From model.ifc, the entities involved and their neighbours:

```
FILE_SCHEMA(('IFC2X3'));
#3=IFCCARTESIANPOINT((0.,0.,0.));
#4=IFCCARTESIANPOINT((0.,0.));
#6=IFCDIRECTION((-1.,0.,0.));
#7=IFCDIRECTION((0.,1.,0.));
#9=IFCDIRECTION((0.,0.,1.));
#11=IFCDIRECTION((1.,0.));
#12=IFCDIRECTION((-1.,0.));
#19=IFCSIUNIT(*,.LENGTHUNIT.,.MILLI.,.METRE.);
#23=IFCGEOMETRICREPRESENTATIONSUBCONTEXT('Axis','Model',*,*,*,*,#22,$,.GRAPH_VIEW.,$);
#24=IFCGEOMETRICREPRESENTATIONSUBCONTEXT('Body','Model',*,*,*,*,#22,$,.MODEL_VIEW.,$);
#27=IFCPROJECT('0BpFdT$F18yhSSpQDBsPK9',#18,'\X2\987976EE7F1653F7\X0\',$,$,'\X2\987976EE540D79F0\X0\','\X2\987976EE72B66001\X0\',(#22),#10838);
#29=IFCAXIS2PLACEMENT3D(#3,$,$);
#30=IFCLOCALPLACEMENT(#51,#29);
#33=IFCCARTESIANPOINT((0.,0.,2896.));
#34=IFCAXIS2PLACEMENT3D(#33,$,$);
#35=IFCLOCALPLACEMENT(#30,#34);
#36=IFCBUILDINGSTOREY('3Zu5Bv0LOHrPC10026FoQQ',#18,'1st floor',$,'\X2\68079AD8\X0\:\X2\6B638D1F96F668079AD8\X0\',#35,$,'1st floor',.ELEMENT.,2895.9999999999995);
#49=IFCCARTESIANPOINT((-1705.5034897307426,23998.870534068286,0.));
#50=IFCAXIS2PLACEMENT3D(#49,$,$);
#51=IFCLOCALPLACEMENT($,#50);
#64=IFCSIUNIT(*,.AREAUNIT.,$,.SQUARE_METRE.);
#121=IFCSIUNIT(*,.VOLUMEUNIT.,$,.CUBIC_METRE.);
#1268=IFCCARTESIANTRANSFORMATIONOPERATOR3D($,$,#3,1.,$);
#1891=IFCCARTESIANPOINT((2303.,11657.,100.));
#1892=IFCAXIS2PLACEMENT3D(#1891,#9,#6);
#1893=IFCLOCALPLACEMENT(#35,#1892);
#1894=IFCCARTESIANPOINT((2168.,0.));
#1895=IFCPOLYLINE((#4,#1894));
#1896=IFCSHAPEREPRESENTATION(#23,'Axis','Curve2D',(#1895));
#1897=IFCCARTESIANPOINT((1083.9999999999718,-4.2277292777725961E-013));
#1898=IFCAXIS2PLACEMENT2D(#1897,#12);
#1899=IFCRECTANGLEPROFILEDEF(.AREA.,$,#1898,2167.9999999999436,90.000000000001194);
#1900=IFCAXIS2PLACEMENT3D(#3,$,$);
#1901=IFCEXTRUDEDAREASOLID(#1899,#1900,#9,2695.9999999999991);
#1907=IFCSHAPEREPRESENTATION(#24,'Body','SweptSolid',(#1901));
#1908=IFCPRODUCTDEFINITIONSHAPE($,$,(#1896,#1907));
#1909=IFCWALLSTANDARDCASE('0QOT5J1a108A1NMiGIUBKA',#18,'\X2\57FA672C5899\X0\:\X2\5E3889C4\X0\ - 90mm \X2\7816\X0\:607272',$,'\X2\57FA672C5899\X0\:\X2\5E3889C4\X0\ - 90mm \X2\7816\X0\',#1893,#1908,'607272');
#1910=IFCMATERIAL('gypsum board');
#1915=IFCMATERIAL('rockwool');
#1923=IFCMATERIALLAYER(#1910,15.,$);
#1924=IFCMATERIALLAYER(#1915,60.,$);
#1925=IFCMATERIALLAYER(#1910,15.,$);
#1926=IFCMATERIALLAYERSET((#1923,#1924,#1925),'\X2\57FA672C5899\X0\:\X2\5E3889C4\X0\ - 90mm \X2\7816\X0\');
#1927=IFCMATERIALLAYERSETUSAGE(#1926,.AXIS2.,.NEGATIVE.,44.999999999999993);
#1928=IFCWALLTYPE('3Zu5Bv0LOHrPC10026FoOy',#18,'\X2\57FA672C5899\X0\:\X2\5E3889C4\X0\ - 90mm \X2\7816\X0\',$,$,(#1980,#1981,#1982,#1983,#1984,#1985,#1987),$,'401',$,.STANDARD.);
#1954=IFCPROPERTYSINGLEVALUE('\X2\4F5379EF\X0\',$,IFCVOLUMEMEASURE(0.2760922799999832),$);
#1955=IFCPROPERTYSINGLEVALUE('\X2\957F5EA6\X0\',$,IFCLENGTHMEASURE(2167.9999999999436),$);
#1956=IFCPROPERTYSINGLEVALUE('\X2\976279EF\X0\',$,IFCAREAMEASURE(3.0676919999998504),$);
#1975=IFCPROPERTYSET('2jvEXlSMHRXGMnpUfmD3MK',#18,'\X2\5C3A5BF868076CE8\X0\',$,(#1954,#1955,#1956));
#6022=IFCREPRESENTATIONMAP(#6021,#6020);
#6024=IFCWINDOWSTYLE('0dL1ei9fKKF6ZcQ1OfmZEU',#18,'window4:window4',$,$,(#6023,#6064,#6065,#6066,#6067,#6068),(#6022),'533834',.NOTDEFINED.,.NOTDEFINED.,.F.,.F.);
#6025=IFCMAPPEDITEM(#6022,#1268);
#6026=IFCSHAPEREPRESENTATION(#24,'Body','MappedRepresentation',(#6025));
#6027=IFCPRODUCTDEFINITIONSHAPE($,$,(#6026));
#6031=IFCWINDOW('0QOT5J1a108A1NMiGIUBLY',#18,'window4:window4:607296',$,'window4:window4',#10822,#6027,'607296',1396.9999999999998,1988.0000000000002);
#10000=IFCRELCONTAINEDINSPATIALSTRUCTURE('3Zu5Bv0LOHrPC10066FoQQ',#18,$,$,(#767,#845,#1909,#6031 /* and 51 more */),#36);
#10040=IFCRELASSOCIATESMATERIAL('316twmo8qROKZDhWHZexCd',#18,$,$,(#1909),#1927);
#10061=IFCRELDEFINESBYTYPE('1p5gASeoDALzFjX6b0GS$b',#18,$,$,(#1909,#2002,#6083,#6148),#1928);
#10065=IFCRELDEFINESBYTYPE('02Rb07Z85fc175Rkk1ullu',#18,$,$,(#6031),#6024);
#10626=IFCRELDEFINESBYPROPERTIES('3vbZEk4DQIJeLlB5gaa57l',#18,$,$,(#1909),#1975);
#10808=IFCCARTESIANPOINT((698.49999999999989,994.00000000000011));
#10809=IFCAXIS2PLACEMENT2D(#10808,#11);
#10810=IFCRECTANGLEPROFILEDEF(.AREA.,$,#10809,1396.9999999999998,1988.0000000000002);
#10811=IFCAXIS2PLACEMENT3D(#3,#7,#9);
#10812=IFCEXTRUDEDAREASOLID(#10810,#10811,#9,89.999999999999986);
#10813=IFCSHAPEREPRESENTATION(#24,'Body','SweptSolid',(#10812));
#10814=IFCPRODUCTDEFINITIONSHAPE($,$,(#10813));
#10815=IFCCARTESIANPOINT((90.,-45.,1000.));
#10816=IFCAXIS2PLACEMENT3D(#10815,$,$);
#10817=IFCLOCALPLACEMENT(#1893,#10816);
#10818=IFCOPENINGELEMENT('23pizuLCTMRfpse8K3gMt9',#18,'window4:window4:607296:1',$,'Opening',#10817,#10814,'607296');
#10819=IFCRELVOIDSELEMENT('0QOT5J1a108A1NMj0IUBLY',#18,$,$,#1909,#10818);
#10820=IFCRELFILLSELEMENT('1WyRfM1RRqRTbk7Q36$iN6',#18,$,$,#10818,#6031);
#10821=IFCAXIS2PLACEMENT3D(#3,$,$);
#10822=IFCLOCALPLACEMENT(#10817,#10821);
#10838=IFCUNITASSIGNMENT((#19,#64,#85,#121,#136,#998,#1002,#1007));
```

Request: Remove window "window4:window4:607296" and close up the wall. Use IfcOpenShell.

```python
import ifcopenshell
import ifcopenshell.api.feature
import ifcopenshell.api.pset
import ifcopenshell.api.root
import ifcopenshell.geom
import ifcopenshell.util.element
import ifcopenshell.util.shape
import ifcopenshell.util.unit

model = ifcopenshell.open("model.ifc")
area_scale = ifcopenshell.util.unit.calculate_unit_scale(model, "AREAUNIT")
volume_scale = ifcopenshell.util.unit.calculate_unit_scale(model, "VOLUMEUNIT")
settings = ifcopenshell.geom.settings()


def volume(element):
    """Net volume in cubic metres, openings subtracted."""
    shape = ifcopenshell.geom.create_shape(settings, element)
    return ifcopenshell.util.shape.get_volume(shape.geometry)


window = model.by_guid("0QOT5J1a108A1NMiGIUBLY")
opening = window.FillsVoids[0].RelatingOpeningElement
wall = opening.VoidsElements[0].RelatingBuildingElement
before = volume(wall)

ifcopenshell.api.root.remove_product(model, product=window)
ifcopenshell.api.feature.remove_feature(model, feature=opening)

after = volume(wall)
thickness = 0.09  # wall thickness in metres

# Update the wall's stored quantities.
pset = model.by_id(ifcopenshell.util.element.get_pset(wall, "尺寸标注", should_inherit=False)["id"])
ifcopenshell.api.pset.edit_pset(model, pset=pset, properties={
    "体积": model.create_entity("IfcVolumeMeasure", after / volume_scale),
    "面积": model.create_entity("IfcAreaMeasure", after / thickness / area_scale),
})

print(f"wall volume {before:.3f} -> {after:.3f} m3")

model.write("model-out.ifc")
```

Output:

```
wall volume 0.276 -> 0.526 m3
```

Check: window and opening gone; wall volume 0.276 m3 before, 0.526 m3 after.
